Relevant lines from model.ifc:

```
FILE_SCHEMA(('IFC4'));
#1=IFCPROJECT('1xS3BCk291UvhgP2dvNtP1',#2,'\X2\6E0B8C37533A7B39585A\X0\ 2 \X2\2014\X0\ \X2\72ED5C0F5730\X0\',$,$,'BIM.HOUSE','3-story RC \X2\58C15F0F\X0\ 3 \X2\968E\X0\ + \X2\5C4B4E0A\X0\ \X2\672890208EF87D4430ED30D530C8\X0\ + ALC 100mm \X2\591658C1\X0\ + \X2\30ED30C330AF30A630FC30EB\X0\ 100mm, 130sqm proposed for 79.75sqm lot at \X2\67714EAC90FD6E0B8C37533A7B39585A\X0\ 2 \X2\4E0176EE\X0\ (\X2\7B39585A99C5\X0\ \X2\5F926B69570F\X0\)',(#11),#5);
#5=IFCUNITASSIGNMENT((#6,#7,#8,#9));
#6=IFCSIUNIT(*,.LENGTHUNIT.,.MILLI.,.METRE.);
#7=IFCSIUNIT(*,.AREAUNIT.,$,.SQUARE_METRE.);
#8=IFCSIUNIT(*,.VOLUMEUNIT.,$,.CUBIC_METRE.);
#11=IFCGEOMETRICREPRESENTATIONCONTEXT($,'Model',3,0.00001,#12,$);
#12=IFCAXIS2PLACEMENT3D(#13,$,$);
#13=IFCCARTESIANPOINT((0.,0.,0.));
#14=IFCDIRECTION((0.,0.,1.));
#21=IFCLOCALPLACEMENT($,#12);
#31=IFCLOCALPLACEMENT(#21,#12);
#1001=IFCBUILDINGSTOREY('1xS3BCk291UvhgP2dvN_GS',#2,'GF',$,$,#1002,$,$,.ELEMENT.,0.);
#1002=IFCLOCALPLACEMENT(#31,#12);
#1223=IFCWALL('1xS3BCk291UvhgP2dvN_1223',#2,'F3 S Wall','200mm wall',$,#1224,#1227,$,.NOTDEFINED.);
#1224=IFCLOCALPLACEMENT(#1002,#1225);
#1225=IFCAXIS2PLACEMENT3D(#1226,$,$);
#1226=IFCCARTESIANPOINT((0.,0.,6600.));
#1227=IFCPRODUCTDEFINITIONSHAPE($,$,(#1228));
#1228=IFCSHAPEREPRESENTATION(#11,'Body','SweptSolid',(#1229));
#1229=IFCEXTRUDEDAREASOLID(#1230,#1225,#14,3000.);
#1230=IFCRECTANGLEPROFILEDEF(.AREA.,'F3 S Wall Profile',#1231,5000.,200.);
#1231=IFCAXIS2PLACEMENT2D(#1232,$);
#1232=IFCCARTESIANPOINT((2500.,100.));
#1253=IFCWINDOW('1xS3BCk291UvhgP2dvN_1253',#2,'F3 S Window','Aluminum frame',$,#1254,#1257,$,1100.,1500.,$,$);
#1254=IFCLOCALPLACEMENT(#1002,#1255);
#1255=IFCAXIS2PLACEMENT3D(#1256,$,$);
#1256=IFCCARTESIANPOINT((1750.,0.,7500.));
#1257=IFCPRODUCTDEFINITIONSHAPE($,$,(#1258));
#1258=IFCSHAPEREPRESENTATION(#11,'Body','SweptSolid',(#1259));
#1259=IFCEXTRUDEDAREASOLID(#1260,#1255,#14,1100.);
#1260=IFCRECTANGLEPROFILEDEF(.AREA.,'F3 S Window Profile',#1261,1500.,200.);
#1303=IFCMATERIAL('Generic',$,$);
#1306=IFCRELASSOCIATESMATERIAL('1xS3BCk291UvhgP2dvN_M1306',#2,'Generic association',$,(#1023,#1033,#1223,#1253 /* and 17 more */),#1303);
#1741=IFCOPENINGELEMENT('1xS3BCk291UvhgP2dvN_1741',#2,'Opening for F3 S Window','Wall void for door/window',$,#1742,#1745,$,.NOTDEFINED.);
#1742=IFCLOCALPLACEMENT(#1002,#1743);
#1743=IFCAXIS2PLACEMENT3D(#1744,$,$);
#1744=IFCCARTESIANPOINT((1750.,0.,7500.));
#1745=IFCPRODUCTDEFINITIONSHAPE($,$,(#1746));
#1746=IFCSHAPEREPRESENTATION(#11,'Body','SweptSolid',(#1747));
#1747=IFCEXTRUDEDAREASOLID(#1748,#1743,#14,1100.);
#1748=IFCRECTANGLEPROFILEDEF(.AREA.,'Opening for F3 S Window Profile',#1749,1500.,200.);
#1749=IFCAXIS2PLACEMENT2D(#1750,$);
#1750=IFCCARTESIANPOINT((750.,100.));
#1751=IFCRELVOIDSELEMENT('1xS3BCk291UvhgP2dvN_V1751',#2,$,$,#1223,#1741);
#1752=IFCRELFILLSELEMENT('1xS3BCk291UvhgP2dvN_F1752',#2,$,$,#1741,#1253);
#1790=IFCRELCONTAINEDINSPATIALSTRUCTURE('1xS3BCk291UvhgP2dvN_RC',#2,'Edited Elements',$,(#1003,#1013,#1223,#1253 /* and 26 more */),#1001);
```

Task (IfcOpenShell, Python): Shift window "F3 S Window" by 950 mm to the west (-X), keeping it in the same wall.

```python
import ifcopenshell
import ifcopenshell.api.geometry
import ifcopenshell.util.placement

model = ifcopenshell.open("model.ifc")

window = model.by_id(1253)
opening = window.FillsVoids[0].RelatingOpeningElement
wall = opening.VoidsElements[0].RelatingBuildingElement

wall_matrix = ifcopenshell.util.placement.get_local_placement(wall.ObjectPlacement)
shift = wall_matrix[:3, 0] * -950.0
before = ifcopenshell.util.placement.get_local_placement(window.ObjectPlacement)[:3, 3].copy()

# The window is not placed relative to its opening, so move both.
for product in (opening, window):
    matrix = ifcopenshell.util.placement.get_local_placement(product.ObjectPlacement)
    matrix[:3, 3] += shift
    ifcopenshell.api.geometry.edit_object_placement(model, product=product, matrix=matrix, is_si=False)

after = ifcopenshell.util.placement.get_local_placement(window.ObjectPlacement)[:3, 3]
print("window moved by", (after - before).round(3) + 0.0)

model.write("model_edited.ifc")
```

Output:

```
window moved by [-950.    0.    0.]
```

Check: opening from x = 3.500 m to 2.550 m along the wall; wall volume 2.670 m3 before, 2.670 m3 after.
